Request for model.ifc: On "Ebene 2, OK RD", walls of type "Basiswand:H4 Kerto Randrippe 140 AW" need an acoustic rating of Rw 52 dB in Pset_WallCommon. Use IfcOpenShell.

First a look at what the model holds.

```python
import ifcopenshell
import ifcopenshell.util.element

model = ifcopenshell.open("model.ifc")
print(model.schema)
storey = next(s for s in model.by_type("IfcBuildingStorey") if s.Name == "Ebene 2, OK RD")
walls = [e for e in ifcopenshell.util.element.get_decomposition(storey) if e.is_a("IfcWall")]
seen = {}
for e in walls:
    element_type = ifcopenshell.util.element.get_type(e)
    key = (element_type.Name if element_type != e and element_type else None, ifcopenshell.util.element.get_pset(e, "Pset_WallCommon", "AcousticRating"))
    seen[key] = seen.get(key, 0) + 1
for (name, value), count in sorted(seen.items(), key=str):
    print(count, "x", name, "|", value)
```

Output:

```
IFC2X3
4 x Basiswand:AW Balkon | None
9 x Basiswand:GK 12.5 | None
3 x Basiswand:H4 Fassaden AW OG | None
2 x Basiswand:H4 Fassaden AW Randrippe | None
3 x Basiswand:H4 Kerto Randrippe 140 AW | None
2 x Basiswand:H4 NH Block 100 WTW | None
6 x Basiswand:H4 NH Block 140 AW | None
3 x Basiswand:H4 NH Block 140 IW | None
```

```python
import ifcopenshell
import ifcopenshell.api.pset
import ifcopenshell.util.element

model = ifcopenshell.open("model.ifc")

storey = next(s for s in model.by_type("IfcBuildingStorey") if s.Name == "Ebene 2, OK RD")
walls = [e for e in ifcopenshell.util.element.get_decomposition(storey) if e.is_a("IfcWall")]

count = 0
for e in walls:
    element_type = ifcopenshell.util.element.get_type(e)
    if element_type in (None, e) or element_type.Name != "Basiswand:H4 Kerto Randrippe 140 AW":
        continue
    # add_pset returns the element's existing set when there is one.
    pset = ifcopenshell.api.pset.add_pset(model, product=e, name="Pset_WallCommon")
    ifcopenshell.api.pset.edit_pset(model, pset=pset, properties={"AcousticRating": "Rw 52 dB"})
    count += 1

print(count, "walls updated")

model.write("model-out.ifc")
```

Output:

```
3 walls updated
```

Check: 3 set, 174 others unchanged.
